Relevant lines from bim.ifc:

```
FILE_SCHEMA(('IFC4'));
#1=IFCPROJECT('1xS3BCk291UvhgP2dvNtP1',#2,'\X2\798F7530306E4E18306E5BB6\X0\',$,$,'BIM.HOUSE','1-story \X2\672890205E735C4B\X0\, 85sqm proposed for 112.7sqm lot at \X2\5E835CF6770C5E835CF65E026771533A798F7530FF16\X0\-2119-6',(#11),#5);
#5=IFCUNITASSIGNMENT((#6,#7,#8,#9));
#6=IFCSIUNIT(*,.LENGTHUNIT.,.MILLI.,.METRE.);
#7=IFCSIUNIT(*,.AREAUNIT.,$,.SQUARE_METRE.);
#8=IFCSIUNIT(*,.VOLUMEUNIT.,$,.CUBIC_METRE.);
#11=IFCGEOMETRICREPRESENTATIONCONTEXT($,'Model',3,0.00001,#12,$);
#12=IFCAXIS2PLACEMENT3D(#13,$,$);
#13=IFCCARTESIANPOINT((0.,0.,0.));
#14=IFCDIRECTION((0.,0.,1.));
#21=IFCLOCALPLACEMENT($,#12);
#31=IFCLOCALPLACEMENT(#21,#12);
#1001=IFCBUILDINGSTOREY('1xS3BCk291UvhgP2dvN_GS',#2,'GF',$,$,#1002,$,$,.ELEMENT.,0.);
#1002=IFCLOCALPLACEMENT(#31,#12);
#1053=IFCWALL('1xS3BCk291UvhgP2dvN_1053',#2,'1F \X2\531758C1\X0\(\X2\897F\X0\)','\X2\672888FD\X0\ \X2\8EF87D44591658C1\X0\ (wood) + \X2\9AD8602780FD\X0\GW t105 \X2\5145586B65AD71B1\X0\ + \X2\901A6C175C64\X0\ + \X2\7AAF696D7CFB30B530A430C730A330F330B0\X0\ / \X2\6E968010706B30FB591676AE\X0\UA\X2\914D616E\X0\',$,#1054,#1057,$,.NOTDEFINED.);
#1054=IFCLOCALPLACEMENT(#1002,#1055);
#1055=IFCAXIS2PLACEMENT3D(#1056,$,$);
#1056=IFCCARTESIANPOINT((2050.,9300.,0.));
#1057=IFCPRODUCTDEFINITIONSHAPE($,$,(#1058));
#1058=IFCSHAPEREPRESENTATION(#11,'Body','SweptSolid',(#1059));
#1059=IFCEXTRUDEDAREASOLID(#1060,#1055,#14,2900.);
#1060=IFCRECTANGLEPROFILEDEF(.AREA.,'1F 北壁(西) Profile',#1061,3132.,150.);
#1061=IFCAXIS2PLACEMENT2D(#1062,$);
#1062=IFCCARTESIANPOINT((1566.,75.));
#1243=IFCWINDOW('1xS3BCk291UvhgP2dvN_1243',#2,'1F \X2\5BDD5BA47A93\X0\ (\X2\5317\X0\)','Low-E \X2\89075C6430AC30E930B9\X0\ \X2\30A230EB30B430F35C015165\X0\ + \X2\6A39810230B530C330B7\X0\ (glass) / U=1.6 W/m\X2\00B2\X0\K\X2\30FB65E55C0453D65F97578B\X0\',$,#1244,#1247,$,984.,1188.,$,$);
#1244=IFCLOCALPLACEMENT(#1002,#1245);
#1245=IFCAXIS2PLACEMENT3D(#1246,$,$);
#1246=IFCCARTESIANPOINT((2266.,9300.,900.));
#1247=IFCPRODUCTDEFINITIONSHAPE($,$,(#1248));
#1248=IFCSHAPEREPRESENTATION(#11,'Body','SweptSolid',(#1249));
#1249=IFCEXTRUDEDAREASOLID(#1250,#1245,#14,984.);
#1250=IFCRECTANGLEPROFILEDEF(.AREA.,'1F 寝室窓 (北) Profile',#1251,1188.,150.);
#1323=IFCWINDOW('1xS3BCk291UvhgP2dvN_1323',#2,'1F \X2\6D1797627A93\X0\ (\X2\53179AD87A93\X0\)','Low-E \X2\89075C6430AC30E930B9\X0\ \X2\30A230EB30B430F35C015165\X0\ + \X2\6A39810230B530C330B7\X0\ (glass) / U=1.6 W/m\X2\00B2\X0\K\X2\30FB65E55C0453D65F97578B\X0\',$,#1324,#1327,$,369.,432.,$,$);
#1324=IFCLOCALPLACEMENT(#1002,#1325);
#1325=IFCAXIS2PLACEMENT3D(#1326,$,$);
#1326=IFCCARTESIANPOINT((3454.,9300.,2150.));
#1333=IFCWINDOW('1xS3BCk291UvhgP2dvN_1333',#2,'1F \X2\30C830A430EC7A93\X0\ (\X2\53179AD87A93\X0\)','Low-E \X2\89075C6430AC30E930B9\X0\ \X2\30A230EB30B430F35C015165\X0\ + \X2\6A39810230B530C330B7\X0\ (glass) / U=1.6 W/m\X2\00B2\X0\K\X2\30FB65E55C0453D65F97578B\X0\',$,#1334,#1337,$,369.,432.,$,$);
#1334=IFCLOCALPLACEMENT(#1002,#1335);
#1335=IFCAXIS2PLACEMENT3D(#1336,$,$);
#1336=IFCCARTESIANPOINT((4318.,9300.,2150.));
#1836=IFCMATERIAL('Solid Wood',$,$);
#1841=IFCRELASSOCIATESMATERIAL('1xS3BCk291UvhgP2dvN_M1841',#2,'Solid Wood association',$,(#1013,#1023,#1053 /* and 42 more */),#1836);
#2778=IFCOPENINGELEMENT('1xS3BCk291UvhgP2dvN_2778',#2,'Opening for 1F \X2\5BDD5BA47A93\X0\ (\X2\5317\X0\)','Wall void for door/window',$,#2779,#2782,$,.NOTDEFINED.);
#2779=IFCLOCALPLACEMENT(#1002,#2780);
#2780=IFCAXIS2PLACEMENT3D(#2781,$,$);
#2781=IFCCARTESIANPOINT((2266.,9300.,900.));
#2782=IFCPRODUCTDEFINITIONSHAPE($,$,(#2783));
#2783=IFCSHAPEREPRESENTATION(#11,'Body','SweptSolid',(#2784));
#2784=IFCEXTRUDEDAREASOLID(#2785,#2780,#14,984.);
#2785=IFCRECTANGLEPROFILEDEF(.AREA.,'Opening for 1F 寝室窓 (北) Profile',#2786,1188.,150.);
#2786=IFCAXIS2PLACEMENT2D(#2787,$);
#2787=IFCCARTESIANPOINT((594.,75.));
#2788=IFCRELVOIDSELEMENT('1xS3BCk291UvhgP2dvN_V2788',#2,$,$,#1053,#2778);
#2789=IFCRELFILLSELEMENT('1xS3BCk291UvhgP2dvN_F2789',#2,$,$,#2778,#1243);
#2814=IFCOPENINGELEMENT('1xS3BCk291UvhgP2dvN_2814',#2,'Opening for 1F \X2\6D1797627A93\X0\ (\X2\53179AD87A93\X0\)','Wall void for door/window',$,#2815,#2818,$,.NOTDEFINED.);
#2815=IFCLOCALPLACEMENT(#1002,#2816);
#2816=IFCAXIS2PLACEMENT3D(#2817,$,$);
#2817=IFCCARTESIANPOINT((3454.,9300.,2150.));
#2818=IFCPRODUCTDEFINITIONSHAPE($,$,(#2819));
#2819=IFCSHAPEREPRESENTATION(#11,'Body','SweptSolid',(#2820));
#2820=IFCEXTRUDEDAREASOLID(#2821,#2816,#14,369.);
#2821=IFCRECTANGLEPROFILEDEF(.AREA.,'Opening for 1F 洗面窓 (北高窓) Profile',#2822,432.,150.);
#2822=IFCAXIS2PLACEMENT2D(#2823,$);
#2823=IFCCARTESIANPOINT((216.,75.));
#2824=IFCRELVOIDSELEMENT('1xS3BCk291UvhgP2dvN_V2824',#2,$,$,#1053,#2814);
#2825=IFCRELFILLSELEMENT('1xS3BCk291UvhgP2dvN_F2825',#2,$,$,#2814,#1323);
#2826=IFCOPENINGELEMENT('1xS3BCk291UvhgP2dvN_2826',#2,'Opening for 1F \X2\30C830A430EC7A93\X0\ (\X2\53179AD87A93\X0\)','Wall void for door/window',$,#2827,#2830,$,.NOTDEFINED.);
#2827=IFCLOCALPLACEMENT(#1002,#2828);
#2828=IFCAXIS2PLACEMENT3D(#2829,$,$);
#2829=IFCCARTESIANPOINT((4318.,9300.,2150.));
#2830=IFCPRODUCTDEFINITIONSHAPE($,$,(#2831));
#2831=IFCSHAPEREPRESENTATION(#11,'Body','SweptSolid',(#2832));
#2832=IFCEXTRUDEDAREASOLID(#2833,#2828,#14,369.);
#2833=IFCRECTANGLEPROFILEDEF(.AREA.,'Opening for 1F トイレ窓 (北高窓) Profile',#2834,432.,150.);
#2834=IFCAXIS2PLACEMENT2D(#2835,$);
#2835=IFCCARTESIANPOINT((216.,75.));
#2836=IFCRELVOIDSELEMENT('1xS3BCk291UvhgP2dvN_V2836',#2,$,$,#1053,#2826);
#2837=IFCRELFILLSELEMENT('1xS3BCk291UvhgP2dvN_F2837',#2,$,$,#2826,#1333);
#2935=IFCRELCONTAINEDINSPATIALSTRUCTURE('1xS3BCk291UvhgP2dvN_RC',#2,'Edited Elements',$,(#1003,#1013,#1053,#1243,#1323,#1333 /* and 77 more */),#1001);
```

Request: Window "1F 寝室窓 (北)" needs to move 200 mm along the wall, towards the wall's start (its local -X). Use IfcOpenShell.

```python
import ifcopenshell
import ifcopenshell.api.geometry
import ifcopenshell.util.placement
import ifcopenshell.util.unit

model = ifcopenshell.open("bim.ifc")
unit_scale = ifcopenshell.util.unit.calculate_unit_scale(model)

window = model.by_id(1243)
opening = window.FillsVoids[0].RelatingOpeningElement
wall = opening.VoidsElements[0].RelatingBuildingElement

wall_matrix = ifcopenshell.util.placement.get_local_placement(wall.ObjectPlacement)
shift = wall_matrix[:3, 0] * -0.2 / unit_scale
before = ifcopenshell.util.placement.get_local_placement(window.ObjectPlacement)[:3, 3].copy()

# The window is not placed relative to its opening, so move both.
for product in (opening, window):
    matrix = ifcopenshell.util.placement.get_local_placement(product.ObjectPlacement)
    matrix[:3, 3] += shift
    ifcopenshell.api.geometry.edit_object_placement(model, product=product, matrix=matrix, is_si=False)

after = ifcopenshell.util.placement.get_local_placement(window.ObjectPlacement)[:3, 3]
print("window moved by", (after - before).round(3) + 0.0)

model.write("bim-out.ifc")
```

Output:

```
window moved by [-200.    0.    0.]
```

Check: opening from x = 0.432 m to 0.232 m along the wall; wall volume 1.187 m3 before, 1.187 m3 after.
